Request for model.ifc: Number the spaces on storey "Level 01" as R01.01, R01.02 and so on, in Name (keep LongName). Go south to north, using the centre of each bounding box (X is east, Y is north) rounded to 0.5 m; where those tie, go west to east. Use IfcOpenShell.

First a look at what the model holds.

```python
import ifcopenshell
import ifcopenshell.util.element
import ifcopenshell.util.placement

model = ifcopenshell.open("model.ifc")
print(model.schema)
storey = next(s for s in model.by_type("IfcBuildingStorey") if s.Name == "Level 01")
spaces = [e for e in ifcopenshell.util.element.get_decomposition(storey) if e.is_a("IfcSpace")]
for e in sorted(spaces, key=lambda e: e.id()):
    origin = ifcopenshell.util.placement.get_local_placement(e.ObjectPlacement)[:3, 3]
    print(e.id(), e.Name, e.LongName, origin.round(2) + 0.0, sep=" | ")
```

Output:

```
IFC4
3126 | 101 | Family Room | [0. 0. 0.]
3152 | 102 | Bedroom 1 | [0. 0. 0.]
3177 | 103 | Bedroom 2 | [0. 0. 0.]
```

```python
import ifcopenshell
import ifcopenshell.geom
import ifcopenshell.util.element
import ifcopenshell.util.shape

model = ifcopenshell.open("model.ifc")
settings = ifcopenshell.geom.settings()
settings.set("use-world-coords", True)


def centre(element):
    shape = ifcopenshell.geom.create_shape(settings, element)
    return ifcopenshell.util.shape.get_bbox_centroid(shape.geometry)


storey = next(s for s in model.by_type("IfcBuildingStorey") if s.Name == "Level 01")
spaces = [e for e in ifcopenshell.util.element.get_decomposition(storey) if e.is_a("IfcSpace")]

# Insertion points can sit at a corner or the storey origin, so sort by the geometry (in metres).
centres = {e: centre(e) for e in spaces}
spaces.sort(key=lambda e: (round(centres[e][1] / 0.5), centres[e][0]))

for i, e in enumerate(spaces, start=1):
    number = f"R01.{i:02d}"
    e.Name = number
    print(e.id(), number)

model.write("model_v2.ifc")
```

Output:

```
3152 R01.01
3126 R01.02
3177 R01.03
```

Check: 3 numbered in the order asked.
